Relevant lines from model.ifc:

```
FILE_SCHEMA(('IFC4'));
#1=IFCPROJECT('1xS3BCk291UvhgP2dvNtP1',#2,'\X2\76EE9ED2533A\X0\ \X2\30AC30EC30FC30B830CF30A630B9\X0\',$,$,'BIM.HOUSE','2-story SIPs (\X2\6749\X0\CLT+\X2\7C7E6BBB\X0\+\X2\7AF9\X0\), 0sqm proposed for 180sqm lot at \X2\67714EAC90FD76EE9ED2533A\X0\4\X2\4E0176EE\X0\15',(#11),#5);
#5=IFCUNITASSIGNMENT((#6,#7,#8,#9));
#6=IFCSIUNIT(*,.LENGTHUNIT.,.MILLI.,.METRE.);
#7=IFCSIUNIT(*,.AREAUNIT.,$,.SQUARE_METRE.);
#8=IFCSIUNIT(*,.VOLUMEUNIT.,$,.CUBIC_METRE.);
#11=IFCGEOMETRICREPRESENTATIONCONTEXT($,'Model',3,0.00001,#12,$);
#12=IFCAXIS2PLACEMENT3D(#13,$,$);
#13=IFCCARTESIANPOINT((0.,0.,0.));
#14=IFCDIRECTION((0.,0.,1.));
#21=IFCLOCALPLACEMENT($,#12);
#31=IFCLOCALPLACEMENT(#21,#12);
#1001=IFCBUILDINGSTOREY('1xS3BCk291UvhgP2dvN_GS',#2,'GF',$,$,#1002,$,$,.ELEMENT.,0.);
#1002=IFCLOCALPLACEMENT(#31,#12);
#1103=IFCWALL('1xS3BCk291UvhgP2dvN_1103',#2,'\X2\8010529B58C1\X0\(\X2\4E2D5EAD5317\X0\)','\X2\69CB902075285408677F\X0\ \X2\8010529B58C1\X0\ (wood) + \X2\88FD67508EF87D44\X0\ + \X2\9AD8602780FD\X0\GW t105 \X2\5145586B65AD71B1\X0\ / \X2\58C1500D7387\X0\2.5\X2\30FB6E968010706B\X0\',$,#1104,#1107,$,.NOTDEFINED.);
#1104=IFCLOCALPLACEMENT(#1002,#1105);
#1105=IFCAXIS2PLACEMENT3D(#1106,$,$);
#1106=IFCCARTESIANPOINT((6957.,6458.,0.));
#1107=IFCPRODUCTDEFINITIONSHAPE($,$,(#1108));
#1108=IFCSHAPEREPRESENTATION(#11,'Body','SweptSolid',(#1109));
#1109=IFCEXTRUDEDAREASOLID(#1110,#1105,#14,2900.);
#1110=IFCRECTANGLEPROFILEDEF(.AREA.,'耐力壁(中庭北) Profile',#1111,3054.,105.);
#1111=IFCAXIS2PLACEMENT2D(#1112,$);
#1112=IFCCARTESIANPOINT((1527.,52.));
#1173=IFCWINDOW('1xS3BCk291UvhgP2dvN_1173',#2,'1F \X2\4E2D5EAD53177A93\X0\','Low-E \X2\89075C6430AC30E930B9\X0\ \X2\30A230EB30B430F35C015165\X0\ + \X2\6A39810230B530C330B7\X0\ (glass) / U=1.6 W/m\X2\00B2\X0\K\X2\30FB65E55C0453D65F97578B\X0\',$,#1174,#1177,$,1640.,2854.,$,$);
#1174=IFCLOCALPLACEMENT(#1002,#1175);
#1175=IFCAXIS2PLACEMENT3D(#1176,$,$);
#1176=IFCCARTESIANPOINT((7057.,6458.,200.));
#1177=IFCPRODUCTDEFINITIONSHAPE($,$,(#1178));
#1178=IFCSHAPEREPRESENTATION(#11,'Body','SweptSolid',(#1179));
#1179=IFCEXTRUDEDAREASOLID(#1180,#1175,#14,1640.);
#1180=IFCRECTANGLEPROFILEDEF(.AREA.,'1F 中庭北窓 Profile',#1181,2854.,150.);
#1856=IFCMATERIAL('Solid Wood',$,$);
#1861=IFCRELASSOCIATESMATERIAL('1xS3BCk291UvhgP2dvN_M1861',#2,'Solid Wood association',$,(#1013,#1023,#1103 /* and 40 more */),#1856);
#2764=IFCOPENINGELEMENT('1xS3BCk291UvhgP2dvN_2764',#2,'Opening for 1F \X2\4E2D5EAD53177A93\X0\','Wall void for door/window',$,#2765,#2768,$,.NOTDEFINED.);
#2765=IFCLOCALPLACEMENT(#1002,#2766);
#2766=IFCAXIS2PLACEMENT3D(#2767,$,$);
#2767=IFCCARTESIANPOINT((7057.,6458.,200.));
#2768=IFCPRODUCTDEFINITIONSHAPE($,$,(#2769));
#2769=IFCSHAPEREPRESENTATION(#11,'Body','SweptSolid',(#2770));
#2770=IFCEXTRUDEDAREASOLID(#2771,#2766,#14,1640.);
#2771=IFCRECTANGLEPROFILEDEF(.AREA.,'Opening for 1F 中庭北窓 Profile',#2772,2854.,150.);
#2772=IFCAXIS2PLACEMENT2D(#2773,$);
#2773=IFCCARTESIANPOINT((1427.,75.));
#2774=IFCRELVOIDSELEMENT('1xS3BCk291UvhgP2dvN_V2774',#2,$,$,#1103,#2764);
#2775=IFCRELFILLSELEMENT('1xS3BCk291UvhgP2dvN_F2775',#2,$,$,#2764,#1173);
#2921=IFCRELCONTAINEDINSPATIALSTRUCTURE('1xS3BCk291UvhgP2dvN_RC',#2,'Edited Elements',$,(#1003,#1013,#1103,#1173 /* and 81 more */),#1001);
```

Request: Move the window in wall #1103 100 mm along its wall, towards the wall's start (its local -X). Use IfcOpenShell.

```python
import ifcopenshell
import ifcopenshell.api.geometry
import ifcopenshell.util.placement
import ifcopenshell.util.unit

model = ifcopenshell.open("model.ifc")
unit_scale = ifcopenshell.util.unit.calculate_unit_scale(model)

window = model.by_id(1173)
opening = window.FillsVoids[0].RelatingOpeningElement
wall = opening.VoidsElements[0].RelatingBuildingElement

wall_matrix = ifcopenshell.util.placement.get_local_placement(wall.ObjectPlacement)
shift = wall_matrix[:3, 0] * -0.1 / unit_scale
before = ifcopenshell.util.placement.get_local_placement(window.ObjectPlacement)[:3, 3].copy()

# The window is not placed relative to its opening, so move both.
for product in (opening, window):
    matrix = ifcopenshell.util.placement.get_local_placement(product.ObjectPlacement)
    matrix[:3, 3] += shift
    ifcopenshell.api.geometry.edit_object_placement(model, product=product, matrix=matrix, is_si=False)

after = ifcopenshell.util.placement.get_local_placement(window.ObjectPlacement)[:3, 3]
print("window moved by", (after - before).round(3) + 0.0)

model.write("model_rev.ifc")
```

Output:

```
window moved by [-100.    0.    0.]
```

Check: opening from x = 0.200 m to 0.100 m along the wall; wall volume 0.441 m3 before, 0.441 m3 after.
